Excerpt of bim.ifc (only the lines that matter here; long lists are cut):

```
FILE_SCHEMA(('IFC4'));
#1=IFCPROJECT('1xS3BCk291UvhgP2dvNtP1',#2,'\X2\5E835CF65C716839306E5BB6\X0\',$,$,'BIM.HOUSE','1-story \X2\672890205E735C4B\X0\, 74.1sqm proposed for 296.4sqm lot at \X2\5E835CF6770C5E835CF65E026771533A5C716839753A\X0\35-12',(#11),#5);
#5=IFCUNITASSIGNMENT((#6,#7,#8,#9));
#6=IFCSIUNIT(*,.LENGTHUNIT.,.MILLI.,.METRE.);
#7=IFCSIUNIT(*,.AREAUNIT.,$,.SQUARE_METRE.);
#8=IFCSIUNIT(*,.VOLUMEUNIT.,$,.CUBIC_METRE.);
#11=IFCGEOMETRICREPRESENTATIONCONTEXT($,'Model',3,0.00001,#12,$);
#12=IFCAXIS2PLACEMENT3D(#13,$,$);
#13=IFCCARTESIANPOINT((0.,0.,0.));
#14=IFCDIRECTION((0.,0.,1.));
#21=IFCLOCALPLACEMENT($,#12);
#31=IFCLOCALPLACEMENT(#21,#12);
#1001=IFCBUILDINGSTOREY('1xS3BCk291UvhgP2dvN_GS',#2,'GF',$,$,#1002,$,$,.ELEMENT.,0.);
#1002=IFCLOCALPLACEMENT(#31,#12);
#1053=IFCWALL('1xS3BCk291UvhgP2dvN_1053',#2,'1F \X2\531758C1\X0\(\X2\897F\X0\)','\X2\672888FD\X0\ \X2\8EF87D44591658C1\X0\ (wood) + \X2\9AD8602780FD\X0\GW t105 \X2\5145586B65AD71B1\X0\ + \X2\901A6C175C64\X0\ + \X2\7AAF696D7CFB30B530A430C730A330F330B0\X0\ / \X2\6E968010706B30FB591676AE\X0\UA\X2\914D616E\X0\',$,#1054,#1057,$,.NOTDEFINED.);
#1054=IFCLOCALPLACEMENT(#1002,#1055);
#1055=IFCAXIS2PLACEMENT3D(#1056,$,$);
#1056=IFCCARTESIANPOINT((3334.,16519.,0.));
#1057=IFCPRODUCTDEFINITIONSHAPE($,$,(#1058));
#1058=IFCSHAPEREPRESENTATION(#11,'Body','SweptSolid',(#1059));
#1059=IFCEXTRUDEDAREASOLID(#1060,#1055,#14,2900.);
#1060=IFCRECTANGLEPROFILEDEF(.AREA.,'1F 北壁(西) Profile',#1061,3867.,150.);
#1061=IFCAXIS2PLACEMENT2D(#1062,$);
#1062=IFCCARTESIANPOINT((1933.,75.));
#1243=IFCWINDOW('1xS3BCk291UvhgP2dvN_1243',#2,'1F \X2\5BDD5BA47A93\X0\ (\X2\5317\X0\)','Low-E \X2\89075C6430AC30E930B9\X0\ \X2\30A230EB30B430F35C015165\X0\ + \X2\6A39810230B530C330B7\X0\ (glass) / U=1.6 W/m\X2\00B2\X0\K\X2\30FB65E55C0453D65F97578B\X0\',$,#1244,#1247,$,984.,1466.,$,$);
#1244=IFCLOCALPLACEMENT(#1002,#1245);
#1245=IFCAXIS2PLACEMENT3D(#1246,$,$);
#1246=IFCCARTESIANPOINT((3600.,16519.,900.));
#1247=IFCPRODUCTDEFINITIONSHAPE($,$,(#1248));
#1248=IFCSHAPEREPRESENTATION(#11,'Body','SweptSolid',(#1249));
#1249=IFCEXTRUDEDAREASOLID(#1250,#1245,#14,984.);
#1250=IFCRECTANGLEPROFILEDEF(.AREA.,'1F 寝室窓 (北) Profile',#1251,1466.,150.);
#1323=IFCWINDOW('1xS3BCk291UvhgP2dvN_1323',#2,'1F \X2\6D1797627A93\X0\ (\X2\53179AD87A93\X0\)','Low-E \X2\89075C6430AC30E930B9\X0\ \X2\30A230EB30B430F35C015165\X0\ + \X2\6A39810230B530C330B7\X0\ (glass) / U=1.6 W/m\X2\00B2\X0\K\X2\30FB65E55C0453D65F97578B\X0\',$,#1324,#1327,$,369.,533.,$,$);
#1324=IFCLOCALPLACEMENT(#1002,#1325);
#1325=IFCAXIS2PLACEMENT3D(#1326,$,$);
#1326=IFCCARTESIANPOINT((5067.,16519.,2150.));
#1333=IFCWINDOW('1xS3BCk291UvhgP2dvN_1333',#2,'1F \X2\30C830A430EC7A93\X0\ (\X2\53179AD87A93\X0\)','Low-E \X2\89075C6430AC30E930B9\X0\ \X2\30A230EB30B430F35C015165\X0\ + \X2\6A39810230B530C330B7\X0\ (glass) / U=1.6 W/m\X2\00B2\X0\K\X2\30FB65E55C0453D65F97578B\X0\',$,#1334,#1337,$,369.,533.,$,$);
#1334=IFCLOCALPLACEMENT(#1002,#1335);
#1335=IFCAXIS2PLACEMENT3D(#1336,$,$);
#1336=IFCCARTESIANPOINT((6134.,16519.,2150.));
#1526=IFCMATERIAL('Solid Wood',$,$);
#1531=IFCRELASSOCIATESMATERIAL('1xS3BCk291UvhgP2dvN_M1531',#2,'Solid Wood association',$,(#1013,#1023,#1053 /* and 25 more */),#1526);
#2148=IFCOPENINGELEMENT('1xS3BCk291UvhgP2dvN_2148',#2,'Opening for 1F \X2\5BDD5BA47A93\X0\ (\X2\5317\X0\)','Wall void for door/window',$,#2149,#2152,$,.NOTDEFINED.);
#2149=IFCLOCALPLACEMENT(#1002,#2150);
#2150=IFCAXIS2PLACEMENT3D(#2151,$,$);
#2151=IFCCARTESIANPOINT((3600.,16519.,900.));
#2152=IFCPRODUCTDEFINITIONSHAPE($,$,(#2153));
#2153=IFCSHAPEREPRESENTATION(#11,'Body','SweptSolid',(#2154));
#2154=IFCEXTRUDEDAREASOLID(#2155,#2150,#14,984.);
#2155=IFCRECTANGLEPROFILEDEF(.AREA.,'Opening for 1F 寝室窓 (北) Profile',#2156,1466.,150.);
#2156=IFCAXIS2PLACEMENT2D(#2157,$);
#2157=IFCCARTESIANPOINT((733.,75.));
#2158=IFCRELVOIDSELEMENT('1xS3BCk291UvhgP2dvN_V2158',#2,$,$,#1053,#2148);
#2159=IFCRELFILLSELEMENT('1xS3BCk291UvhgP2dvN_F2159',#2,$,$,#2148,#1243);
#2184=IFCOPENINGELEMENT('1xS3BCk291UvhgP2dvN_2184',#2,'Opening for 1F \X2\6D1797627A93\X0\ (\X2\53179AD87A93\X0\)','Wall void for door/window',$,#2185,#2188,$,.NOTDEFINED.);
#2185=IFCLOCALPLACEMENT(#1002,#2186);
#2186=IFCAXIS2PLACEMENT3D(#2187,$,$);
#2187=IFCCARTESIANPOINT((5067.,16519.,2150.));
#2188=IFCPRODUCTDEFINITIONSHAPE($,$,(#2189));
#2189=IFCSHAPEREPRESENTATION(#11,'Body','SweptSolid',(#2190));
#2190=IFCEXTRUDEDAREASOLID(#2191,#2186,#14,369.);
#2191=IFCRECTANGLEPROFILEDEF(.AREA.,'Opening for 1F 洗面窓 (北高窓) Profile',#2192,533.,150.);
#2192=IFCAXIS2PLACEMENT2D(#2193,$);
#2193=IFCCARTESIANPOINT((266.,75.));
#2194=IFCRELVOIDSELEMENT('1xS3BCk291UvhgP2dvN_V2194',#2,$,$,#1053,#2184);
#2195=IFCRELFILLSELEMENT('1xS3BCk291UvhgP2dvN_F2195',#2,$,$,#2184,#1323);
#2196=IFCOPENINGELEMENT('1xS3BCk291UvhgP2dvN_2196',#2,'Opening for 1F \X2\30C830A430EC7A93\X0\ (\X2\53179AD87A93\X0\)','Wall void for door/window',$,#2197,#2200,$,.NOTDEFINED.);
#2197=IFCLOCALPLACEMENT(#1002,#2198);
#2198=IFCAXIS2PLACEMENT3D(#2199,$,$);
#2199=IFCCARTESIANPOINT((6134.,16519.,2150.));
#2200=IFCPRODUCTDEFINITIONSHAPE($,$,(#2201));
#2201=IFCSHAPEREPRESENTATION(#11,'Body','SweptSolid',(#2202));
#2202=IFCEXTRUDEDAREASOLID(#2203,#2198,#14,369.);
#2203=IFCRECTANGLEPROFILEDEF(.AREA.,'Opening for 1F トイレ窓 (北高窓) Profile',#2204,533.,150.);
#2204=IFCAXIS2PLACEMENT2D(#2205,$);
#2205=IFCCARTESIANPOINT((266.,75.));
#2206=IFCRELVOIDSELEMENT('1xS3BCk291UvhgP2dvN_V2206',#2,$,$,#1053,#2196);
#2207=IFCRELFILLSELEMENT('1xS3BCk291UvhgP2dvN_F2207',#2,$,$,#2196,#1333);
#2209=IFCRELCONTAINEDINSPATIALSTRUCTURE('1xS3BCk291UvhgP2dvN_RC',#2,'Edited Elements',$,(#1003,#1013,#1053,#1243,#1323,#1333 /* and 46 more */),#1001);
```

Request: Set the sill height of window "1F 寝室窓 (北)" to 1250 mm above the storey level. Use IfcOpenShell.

```python
import numpy as np
import ifcopenshell
import ifcopenshell.api.geometry
import ifcopenshell.geom
import ifcopenshell.util.element
import ifcopenshell.util.placement
import ifcopenshell.util.shape
import ifcopenshell.util.unit

model = ifcopenshell.open("bim.ifc")
unit_scale = ifcopenshell.util.unit.calculate_unit_scale(model)

window = model.by_guid("1xS3BCk291UvhgP2dvN_1243")
opening = window.FillsVoids[0].RelatingOpeningElement
storey = ifcopenshell.util.element.get_container(window, ifc_class="IfcBuildingStorey")
level = ifcopenshell.util.placement.get_local_placement(storey.ObjectPlacement)[2, 3]

# The opening's origin need not be at the sill, so measure its lowest point.
shape = ifcopenshell.geom.create_shape(ifcopenshell.geom.settings(), opening)
bottom = ifcopenshell.util.shape.get_shape_bottom_elevation(shape, shape.geometry) / unit_scale
dz = level + 1.25 / unit_scale - bottom

shift = np.array([0.0, 0.0, dz])
# The window is not placed relative to its opening, so move both.
for product in (opening, window):
    matrix = ifcopenshell.util.placement.get_local_placement(product.ObjectPlacement)
    matrix[:3, 3] += shift
    ifcopenshell.api.geometry.edit_object_placement(model, product=product, matrix=matrix, is_si=False)

print(f"moved by {dz * unit_scale:+.3f} m")

model.write("bim_updated.ifc")
```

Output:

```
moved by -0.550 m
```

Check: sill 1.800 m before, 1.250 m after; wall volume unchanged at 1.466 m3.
